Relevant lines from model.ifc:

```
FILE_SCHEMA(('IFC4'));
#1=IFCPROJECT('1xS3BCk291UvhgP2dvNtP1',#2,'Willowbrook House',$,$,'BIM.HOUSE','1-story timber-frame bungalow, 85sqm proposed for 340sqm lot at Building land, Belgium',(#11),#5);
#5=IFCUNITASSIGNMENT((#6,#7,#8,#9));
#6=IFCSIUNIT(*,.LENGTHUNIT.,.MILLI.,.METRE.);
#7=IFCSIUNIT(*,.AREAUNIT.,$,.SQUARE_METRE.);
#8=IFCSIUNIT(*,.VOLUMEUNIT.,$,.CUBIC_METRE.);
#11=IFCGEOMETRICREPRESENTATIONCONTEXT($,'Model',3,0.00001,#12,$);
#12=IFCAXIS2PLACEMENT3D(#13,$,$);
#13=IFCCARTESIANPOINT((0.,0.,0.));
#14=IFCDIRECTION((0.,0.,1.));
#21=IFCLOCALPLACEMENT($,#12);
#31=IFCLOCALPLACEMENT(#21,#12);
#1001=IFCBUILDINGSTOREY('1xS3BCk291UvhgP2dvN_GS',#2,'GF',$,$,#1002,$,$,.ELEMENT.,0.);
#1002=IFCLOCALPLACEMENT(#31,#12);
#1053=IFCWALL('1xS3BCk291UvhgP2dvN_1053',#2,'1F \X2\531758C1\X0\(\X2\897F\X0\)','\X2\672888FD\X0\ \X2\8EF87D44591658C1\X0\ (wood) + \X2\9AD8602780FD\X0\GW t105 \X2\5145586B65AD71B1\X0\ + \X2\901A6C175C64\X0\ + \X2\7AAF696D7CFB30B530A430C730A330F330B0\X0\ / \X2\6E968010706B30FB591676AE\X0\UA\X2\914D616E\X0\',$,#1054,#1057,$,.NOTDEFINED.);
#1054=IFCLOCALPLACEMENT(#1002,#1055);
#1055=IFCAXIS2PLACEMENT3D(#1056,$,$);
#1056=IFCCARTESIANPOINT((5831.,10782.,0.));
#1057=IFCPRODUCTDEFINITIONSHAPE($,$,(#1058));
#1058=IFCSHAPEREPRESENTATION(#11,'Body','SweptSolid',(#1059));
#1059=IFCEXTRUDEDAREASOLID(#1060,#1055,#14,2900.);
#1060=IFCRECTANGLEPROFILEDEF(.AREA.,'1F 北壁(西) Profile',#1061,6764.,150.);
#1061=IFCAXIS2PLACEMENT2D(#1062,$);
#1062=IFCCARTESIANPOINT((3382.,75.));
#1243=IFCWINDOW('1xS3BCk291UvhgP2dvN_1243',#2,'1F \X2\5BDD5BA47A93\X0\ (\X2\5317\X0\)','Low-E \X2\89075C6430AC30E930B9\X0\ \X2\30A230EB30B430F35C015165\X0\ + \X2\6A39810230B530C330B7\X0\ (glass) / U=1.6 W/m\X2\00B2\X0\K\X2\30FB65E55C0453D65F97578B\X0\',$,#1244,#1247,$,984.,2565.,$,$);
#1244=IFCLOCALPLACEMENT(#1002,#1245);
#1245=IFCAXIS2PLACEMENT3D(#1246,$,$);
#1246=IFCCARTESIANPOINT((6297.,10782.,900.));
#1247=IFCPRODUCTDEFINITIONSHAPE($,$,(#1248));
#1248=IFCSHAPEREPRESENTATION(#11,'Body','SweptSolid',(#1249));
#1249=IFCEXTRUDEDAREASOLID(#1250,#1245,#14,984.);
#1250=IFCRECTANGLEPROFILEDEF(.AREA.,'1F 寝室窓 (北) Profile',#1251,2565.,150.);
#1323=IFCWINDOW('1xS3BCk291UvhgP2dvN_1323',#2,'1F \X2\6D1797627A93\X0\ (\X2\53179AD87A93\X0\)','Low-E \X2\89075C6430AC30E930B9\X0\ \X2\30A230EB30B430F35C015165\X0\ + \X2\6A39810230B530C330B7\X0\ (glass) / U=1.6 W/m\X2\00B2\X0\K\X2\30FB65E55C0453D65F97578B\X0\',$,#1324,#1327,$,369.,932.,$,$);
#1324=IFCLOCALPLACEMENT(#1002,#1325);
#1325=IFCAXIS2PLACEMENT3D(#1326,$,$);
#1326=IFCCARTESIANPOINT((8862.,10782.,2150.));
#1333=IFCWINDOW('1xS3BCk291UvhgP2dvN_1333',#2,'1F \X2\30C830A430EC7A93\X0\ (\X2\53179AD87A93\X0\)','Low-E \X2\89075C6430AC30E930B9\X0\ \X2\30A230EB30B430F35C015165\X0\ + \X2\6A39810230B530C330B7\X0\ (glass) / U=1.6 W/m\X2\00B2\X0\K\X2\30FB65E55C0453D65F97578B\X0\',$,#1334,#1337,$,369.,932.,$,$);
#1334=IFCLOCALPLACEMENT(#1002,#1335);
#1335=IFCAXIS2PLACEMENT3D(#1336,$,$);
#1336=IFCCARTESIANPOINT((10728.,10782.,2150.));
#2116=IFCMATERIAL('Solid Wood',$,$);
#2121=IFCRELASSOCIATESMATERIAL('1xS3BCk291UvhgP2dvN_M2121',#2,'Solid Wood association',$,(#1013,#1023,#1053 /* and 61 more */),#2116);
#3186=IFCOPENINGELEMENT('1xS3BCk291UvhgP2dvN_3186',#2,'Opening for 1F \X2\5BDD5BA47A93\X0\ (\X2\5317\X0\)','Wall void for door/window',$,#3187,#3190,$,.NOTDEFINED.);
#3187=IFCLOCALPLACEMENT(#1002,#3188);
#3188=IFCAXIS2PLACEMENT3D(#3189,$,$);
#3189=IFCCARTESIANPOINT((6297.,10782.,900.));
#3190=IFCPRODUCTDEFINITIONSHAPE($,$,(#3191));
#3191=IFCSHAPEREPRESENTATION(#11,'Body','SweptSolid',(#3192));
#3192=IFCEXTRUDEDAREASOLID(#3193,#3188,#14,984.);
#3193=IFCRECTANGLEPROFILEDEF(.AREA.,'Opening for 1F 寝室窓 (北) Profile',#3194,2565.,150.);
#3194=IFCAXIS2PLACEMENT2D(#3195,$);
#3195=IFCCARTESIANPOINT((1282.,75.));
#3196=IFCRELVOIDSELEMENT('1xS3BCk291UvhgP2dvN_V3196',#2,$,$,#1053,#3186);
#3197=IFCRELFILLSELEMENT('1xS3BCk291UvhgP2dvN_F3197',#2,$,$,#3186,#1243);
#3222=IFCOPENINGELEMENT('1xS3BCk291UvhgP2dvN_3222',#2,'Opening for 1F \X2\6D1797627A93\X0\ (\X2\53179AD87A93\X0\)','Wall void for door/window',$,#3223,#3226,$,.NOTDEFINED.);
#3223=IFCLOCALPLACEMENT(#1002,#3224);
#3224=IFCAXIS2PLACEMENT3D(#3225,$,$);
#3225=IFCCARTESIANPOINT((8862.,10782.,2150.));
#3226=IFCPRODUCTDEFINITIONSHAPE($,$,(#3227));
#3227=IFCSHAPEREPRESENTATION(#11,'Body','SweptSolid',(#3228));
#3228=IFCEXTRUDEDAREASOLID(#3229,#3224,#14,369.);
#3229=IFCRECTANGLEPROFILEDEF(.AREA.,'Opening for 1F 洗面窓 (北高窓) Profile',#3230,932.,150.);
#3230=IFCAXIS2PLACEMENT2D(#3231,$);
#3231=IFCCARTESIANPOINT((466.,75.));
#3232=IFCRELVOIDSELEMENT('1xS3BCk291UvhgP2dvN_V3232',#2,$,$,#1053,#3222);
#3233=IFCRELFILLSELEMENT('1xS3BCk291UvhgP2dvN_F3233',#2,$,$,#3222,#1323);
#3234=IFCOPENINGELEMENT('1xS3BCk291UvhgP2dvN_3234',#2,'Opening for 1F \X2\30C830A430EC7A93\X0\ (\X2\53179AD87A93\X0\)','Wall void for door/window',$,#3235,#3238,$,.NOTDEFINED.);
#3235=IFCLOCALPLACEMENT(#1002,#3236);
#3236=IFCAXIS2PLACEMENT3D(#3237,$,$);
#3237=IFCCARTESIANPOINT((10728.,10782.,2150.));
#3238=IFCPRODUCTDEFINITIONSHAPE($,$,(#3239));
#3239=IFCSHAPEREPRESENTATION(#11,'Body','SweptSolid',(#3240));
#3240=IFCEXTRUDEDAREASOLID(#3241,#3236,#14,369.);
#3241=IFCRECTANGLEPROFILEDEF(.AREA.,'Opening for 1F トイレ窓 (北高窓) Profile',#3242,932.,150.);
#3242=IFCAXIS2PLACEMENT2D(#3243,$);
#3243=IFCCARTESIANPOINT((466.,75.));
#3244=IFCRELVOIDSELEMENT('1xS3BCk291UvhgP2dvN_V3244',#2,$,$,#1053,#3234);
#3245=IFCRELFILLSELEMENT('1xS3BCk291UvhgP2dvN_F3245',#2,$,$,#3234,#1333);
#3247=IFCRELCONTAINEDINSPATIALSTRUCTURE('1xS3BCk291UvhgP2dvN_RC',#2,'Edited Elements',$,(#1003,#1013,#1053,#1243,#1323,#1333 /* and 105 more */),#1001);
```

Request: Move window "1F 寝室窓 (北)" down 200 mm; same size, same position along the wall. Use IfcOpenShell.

```python
import numpy as np
import ifcopenshell
import ifcopenshell.api.geometry
import ifcopenshell.util.placement
import ifcopenshell.util.unit

model = ifcopenshell.open("model.ifc")
unit_scale = ifcopenshell.util.unit.calculate_unit_scale(model)

window = model.by_guid("1xS3BCk291UvhgP2dvN_1243")
opening = window.FillsVoids[0].RelatingOpeningElement
dz = -0.2 / unit_scale

shift = np.array([0.0, 0.0, dz])
# The window is not placed relative to its opening, so move both.
for product in (opening, window):
    matrix = ifcopenshell.util.placement.get_local_placement(product.ObjectPlacement)
    matrix[:3, 3] += shift
    ifcopenshell.api.geometry.edit_object_placement(model, product=product, matrix=matrix, is_si=False)

print(f"moved by {dz * unit_scale:+.3f} m")

model.write("model_v2.ifc")
```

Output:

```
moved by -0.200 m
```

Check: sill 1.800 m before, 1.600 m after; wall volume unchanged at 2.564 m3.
